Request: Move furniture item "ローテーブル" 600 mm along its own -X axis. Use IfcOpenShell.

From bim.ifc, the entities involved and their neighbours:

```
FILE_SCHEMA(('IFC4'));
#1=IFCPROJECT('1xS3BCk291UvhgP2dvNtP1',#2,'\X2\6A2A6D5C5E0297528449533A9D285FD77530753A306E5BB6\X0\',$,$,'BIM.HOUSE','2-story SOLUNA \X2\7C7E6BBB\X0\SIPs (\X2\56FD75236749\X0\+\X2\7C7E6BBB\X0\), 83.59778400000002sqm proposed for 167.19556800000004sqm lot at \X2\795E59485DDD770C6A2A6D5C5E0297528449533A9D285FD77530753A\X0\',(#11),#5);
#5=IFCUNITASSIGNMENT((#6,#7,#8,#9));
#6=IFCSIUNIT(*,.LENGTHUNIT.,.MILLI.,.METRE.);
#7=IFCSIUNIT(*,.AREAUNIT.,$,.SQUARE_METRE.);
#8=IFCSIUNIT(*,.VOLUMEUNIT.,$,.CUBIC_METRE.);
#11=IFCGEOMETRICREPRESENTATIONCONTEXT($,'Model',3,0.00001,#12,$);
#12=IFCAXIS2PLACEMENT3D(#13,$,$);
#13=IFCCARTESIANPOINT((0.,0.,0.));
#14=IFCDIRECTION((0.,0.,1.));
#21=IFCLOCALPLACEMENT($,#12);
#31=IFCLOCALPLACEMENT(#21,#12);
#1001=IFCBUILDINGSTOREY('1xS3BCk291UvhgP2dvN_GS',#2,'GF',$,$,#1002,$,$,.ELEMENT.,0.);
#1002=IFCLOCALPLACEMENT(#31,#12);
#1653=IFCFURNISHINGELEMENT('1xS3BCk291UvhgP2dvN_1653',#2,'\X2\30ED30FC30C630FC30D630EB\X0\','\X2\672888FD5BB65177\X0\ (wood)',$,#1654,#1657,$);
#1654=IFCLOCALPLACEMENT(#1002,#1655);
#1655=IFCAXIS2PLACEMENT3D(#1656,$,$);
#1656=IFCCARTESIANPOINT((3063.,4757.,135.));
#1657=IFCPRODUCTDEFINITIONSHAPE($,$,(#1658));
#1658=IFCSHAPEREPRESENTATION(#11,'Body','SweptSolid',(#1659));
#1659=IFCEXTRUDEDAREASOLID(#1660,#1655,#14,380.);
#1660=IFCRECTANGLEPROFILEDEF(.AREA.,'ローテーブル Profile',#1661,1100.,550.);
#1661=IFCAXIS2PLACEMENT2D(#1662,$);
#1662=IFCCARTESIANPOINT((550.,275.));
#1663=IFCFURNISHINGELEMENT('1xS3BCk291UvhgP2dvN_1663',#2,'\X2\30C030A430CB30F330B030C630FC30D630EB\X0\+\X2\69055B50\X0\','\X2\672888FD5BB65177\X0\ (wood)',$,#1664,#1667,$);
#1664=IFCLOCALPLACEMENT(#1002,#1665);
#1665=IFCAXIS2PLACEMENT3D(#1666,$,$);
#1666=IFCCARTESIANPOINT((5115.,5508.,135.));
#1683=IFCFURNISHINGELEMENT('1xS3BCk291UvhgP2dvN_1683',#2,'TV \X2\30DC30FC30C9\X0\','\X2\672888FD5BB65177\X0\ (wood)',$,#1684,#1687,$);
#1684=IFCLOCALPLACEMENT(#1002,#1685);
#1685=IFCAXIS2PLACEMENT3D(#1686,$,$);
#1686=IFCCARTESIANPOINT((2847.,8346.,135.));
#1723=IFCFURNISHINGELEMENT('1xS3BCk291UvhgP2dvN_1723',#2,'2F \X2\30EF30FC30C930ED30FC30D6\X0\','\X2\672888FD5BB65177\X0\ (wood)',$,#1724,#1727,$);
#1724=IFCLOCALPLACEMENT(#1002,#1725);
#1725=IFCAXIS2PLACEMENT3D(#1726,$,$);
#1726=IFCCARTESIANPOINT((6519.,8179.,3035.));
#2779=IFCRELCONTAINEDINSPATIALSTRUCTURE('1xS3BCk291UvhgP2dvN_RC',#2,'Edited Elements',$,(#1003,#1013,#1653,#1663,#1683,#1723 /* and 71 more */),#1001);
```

```python
import ifcopenshell
import ifcopenshell.api.geometry
import ifcopenshell.util.placement
import ifcopenshell.util.unit

model = ifcopenshell.open("bim.ifc")
unit_scale = ifcopenshell.util.unit.calculate_unit_scale(model)

item = model.by_id(1653)
matrix = ifcopenshell.util.placement.get_local_placement(item.ObjectPlacement)
matrix[:3, 3] -= matrix[:3, 0] * 0.6 / unit_scale
ifcopenshell.api.geometry.edit_object_placement(model, product=item, matrix=matrix, is_si=False)

print(ifcopenshell.util.placement.get_local_placement(item.ObjectPlacement).round(3) + 0.0)

model.write("bim_edited.ifc")
```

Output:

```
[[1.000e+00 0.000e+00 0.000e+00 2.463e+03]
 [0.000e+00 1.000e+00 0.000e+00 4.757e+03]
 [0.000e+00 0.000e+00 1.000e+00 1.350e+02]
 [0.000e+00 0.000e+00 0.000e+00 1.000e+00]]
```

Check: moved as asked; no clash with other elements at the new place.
